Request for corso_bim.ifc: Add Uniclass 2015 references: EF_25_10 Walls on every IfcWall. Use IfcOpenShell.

First a look at what the model holds.

```python
import ifcopenshell

model = ifcopenshell.open("corso_bim.ifc")
print(model.schema)
print("classifications:", [c.Name for c in model.by_type("IfcClassification")])
for ifc_class in ("IfcDoor", "IfcRoof", "IfcStair", "IfcWall", "IfcWindow"):
    print(ifc_class, len(model.by_type(ifc_class)))
```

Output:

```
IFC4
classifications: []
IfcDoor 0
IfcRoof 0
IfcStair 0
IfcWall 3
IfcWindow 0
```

```python
import ifcopenshell
import ifcopenshell.api.classification

model = ifcopenshell.open("corso_bim.ifc")

system = ifcopenshell.api.classification.add_classification(model, classification="Uniclass 2015")

codes = {
    "IfcWall": ("EF_25_10", "Walls"),
}
for ifc_class, (code, name) in codes.items():
    products = model.by_type(ifc_class)
    ifcopenshell.api.classification.add_reference(
        model, products=products, classification=system, identification=code, name=name
    )
    print(code, len(products))

model.write("corso_bim_edited.ifc")
```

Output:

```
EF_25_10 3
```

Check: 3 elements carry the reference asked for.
